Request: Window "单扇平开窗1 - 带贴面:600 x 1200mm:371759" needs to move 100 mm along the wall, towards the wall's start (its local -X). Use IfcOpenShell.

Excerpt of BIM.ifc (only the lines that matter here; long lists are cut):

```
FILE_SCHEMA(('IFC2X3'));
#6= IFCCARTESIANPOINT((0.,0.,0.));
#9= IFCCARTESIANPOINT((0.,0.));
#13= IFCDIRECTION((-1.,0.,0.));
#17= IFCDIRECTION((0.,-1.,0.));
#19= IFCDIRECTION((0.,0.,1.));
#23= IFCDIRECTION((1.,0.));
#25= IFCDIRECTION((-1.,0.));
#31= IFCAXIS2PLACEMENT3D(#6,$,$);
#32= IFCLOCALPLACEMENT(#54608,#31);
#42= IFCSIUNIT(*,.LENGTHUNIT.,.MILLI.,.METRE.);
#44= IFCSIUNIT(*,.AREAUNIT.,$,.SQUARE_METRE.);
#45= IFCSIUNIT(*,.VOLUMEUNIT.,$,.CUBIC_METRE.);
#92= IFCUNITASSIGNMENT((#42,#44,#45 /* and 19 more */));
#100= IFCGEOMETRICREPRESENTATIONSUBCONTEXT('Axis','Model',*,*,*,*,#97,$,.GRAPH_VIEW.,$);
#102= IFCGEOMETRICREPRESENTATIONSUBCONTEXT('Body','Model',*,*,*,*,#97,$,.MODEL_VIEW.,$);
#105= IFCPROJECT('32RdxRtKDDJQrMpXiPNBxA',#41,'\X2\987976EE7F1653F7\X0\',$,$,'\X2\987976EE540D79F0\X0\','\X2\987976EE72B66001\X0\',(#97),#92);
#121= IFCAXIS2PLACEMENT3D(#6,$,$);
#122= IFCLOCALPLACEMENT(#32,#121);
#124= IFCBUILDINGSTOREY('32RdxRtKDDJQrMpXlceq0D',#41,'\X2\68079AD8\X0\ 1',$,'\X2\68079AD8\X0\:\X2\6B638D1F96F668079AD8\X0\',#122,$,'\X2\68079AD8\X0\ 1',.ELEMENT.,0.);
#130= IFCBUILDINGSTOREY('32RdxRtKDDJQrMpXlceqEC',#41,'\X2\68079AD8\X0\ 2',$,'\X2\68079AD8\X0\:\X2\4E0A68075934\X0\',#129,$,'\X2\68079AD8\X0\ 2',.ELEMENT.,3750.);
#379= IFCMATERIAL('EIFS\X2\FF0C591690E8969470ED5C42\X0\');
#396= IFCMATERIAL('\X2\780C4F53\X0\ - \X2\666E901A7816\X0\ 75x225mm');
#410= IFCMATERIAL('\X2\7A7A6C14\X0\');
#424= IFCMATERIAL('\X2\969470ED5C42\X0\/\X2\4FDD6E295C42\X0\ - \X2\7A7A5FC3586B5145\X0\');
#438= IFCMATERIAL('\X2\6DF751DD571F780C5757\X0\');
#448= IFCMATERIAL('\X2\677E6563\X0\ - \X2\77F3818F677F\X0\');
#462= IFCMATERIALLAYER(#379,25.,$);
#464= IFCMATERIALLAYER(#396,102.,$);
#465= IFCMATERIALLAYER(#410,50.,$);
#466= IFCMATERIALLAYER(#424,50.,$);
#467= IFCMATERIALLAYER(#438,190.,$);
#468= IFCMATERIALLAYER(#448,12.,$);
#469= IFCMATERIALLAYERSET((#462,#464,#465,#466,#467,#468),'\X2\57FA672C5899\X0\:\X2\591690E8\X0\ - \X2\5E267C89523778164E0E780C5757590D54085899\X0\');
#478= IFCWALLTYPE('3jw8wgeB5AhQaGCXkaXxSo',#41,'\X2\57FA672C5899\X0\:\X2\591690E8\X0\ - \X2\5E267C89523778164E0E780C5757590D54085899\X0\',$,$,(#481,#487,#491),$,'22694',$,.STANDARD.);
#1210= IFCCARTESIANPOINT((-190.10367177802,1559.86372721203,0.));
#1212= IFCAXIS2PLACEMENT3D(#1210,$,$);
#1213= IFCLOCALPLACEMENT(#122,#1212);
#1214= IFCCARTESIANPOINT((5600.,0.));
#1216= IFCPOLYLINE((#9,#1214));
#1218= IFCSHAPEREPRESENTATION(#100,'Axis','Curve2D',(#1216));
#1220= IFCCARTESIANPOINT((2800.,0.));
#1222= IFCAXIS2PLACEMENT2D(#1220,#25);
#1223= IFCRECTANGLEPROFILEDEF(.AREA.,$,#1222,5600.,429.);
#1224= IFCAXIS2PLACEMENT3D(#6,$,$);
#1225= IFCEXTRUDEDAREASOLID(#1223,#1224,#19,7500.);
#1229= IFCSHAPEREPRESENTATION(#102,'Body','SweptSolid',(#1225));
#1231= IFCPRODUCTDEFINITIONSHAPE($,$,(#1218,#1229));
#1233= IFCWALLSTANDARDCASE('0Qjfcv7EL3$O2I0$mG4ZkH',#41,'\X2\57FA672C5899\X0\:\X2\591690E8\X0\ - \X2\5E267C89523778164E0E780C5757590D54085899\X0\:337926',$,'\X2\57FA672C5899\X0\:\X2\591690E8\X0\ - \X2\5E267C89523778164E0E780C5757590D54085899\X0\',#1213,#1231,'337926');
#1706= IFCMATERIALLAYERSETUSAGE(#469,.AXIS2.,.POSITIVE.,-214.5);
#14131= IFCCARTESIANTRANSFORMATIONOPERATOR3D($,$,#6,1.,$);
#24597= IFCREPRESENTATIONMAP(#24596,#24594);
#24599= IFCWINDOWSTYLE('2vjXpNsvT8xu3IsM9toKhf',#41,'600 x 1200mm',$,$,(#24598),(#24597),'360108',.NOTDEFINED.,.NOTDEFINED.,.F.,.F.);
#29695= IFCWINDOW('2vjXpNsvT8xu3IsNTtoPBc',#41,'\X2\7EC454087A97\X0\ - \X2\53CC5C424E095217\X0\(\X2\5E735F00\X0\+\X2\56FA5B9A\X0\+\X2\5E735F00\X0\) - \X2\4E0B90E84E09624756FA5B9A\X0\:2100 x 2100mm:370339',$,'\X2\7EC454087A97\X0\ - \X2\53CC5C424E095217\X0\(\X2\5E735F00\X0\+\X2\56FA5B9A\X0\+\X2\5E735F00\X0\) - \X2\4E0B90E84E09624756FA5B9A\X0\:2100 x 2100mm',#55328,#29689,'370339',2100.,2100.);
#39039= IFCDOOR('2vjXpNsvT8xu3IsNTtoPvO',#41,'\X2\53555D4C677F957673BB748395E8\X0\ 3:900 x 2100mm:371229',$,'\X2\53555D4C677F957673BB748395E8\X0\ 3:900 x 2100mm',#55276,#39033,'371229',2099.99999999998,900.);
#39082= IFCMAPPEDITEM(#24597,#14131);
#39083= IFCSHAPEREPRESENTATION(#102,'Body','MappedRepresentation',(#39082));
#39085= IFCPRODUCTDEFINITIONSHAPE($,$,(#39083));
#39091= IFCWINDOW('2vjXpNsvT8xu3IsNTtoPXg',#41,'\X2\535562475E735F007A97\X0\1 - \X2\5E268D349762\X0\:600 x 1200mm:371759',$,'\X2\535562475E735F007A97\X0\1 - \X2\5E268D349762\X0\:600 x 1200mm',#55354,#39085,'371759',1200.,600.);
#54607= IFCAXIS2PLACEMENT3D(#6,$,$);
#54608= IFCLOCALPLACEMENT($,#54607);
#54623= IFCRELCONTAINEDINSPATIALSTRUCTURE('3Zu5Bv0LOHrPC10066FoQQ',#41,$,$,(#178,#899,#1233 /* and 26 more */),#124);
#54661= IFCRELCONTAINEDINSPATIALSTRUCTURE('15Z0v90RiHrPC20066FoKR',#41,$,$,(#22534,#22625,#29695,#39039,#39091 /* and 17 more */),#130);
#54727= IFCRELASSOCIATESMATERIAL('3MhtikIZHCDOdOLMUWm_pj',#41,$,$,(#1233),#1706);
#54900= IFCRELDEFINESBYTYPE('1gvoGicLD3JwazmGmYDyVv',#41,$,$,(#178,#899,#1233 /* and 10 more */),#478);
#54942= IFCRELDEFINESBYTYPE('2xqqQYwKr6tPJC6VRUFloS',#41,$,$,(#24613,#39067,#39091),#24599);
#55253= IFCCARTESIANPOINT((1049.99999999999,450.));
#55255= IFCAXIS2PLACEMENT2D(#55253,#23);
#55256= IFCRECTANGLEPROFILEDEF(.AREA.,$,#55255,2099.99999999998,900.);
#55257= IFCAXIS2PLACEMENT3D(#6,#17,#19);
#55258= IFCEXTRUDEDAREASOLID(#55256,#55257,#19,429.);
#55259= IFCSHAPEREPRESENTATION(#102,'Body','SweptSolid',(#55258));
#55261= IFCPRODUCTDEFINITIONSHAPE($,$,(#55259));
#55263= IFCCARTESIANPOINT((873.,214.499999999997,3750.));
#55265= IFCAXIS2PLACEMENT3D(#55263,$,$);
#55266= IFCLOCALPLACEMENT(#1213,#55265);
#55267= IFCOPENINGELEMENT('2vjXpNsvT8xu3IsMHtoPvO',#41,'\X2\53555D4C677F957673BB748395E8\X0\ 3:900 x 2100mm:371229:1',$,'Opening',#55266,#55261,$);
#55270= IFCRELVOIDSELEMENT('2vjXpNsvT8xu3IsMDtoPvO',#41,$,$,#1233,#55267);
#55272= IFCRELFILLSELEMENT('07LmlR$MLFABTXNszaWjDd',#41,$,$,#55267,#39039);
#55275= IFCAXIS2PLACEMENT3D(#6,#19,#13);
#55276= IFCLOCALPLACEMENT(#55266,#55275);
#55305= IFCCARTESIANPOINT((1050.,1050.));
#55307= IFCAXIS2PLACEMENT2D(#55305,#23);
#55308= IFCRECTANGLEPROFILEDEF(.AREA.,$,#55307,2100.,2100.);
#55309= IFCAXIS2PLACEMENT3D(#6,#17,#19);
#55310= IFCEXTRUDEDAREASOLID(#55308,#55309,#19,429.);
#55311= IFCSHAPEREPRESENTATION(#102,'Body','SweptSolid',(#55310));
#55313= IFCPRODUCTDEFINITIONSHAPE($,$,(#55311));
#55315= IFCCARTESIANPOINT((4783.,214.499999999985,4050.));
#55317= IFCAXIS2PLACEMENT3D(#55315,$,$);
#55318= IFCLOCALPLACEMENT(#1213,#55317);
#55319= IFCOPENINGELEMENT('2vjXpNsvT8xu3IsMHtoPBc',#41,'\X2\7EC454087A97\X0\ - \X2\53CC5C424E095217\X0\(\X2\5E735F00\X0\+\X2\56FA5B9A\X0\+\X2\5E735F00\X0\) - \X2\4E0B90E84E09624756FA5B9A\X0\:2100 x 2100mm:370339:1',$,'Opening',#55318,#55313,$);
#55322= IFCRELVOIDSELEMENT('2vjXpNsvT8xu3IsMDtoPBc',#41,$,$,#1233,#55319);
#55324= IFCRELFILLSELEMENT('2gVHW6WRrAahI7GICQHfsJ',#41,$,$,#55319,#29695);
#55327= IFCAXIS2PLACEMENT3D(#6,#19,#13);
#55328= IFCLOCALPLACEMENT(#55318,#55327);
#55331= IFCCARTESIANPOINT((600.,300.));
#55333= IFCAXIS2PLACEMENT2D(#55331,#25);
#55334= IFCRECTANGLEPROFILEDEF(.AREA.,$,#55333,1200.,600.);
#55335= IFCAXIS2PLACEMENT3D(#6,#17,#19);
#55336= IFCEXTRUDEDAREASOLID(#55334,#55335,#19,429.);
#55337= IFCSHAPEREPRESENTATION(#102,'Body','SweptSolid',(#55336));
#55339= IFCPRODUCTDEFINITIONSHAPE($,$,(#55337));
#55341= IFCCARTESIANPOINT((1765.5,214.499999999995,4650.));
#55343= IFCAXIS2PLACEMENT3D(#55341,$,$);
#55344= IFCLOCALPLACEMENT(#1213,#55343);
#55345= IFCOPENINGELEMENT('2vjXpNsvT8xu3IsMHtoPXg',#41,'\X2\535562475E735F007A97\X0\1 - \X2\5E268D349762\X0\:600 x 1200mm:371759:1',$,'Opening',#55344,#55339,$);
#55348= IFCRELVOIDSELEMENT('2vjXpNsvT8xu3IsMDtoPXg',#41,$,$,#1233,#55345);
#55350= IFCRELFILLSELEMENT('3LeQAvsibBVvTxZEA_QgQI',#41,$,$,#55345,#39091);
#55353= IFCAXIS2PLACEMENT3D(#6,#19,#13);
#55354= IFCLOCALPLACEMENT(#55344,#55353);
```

```python
import ifcopenshell
import ifcopenshell.api.geometry
import ifcopenshell.util.placement
import ifcopenshell.util.unit

model = ifcopenshell.open("BIM.ifc")
unit_scale = ifcopenshell.util.unit.calculate_unit_scale(model)

window = model.by_guid("2vjXpNsvT8xu3IsNTtoPXg")
opening = window.FillsVoids[0].RelatingOpeningElement
wall = opening.VoidsElements[0].RelatingBuildingElement

wall_matrix = ifcopenshell.util.placement.get_local_placement(wall.ObjectPlacement)
shift = wall_matrix[:3, 0] * -0.1 / unit_scale
before = ifcopenshell.util.placement.get_local_placement(window.ObjectPlacement)[:3, 3].copy()

# The window is placed relative to its opening, so it follows when the opening moves.
matrix = ifcopenshell.util.placement.get_local_placement(opening.ObjectPlacement)
matrix[:3, 3] += shift
ifcopenshell.api.geometry.edit_object_placement(
    model, product=opening, matrix=matrix, is_si=False, should_transform_children=True
)

after = ifcopenshell.util.placement.get_local_placement(window.ObjectPlacement)[:3, 3]
print("window moved by", (after - before).round(3) + 0.0)

model.write("BIM_v2.ifc")
```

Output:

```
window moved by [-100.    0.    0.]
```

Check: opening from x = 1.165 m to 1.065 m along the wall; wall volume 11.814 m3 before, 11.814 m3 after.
